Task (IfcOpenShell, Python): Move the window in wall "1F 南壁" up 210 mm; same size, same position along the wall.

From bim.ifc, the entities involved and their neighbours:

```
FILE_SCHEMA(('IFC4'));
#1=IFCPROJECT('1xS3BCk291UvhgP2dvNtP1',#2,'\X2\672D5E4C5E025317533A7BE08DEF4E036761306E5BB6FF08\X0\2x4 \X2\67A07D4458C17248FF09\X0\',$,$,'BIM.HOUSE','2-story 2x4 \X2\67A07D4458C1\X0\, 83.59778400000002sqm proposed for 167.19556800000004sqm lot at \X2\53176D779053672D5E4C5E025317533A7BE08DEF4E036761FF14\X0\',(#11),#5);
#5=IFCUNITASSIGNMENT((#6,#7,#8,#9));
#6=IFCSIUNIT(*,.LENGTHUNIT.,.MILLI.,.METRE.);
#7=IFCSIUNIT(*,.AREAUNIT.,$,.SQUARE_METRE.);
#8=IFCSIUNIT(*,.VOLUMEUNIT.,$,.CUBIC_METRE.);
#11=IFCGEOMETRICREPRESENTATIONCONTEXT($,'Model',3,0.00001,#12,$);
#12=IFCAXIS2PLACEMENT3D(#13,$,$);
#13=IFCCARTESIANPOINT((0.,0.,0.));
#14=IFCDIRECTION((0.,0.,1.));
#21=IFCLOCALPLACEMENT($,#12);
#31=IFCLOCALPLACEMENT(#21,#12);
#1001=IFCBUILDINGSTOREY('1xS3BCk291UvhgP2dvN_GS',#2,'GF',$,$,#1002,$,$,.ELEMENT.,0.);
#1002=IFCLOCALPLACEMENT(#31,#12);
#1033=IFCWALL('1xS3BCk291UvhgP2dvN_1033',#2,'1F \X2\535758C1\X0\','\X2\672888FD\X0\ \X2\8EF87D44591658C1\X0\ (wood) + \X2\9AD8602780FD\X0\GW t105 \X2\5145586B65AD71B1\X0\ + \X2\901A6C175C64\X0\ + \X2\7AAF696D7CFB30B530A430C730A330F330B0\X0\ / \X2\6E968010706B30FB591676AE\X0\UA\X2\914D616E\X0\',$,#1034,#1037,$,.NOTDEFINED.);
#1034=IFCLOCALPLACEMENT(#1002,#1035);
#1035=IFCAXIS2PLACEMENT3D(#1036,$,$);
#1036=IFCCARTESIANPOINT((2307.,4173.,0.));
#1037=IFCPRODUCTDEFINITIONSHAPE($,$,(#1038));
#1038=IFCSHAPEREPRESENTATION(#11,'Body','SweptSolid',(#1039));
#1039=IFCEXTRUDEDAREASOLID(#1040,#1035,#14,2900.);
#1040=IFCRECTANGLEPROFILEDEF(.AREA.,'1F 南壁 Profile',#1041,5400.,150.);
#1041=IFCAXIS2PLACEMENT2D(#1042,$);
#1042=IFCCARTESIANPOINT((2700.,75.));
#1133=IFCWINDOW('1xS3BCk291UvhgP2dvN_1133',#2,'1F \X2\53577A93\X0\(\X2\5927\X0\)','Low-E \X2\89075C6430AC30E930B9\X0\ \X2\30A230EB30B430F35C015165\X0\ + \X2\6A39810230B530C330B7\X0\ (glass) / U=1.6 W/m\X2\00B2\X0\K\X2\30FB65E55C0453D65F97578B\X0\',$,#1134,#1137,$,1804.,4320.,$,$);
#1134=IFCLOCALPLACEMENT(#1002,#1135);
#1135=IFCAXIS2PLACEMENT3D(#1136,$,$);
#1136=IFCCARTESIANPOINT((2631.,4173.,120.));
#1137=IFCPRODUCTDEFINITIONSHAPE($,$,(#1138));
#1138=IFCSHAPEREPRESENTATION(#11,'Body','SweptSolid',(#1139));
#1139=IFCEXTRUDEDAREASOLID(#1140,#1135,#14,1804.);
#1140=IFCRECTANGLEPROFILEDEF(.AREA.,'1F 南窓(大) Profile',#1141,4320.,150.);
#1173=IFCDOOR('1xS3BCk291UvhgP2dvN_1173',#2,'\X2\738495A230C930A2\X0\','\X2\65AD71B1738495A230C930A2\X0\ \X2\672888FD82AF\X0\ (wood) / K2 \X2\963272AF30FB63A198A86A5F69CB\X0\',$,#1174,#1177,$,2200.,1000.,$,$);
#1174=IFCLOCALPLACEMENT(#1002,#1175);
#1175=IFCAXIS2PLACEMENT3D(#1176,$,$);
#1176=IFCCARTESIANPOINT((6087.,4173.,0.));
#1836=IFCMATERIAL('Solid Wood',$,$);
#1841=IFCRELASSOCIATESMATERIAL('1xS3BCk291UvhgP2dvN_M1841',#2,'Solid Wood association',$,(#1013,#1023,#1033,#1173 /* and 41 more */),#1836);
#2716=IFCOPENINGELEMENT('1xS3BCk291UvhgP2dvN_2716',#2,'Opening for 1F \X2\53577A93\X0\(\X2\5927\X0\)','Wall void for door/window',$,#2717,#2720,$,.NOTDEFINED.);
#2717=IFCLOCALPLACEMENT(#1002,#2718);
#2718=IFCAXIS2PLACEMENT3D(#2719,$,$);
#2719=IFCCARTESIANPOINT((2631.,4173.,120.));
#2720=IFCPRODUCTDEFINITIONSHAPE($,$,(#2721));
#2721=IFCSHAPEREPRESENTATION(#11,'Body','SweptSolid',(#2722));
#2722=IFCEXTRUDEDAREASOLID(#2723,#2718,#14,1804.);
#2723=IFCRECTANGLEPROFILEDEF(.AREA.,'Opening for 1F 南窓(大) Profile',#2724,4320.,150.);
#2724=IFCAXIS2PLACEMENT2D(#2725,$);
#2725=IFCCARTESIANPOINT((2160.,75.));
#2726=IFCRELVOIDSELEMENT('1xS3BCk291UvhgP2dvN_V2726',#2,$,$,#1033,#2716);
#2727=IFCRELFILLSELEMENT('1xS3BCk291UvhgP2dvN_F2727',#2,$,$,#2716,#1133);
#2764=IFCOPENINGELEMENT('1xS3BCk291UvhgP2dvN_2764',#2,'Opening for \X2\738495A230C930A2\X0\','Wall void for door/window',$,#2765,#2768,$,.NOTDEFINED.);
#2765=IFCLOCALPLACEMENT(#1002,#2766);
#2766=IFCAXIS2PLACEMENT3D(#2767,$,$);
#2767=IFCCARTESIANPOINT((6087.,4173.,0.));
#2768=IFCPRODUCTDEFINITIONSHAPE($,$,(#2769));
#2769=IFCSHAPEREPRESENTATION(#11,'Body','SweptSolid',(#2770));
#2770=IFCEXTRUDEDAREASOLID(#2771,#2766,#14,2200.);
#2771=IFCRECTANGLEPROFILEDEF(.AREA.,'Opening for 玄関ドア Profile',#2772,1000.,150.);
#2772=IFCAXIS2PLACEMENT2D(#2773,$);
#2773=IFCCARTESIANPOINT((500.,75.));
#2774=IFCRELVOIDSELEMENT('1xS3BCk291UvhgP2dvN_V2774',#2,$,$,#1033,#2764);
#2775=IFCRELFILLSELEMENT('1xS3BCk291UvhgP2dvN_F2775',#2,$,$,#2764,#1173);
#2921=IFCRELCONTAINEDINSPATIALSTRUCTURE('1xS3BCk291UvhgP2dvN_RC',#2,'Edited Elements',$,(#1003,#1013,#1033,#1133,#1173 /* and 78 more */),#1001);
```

```python
import numpy as np
import ifcopenshell
import ifcopenshell.api.geometry
import ifcopenshell.util.placement
import ifcopenshell.util.unit

model = ifcopenshell.open("bim.ifc")
unit_scale = ifcopenshell.util.unit.calculate_unit_scale(model)

window = model.by_id(1133)
opening = window.FillsVoids[0].RelatingOpeningElement
dz = 210.0

shift = np.array([0.0, 0.0, dz])
# The window is not placed relative to its opening, so move both.
for product in (opening, window):
    matrix = ifcopenshell.util.placement.get_local_placement(product.ObjectPlacement)
    matrix[:3, 3] += shift
    ifcopenshell.api.geometry.edit_object_placement(model, product=product, matrix=matrix, is_si=False)

print(f"moved by {dz * unit_scale:+.3f} m")

model.write("bim_v2.ifc")
```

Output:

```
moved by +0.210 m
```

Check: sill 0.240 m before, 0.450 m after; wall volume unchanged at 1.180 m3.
